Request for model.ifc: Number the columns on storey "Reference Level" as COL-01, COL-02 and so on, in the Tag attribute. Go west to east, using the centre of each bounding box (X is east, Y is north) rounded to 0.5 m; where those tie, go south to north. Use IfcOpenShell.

First a look at what the model holds.

```python
import ifcopenshell
import ifcopenshell.util.element
import ifcopenshell.util.placement

model = ifcopenshell.open("model.ifc")
print(model.schema)
storey = next(s for s in model.by_type("IfcBuildingStorey") if s.Name == "Reference Level")
columns = [e for e in ifcopenshell.util.element.get_decomposition(storey) if e.is_a("IfcColumn")]
for e in sorted(columns, key=lambda e: e.id()):
    origin = ifcopenshell.util.placement.get_local_placement(e.ObjectPlacement)[:3, 3]
    print(e.id(), e.Tag, e.Name, origin.round(2) + 0.0, sep=" | ")
```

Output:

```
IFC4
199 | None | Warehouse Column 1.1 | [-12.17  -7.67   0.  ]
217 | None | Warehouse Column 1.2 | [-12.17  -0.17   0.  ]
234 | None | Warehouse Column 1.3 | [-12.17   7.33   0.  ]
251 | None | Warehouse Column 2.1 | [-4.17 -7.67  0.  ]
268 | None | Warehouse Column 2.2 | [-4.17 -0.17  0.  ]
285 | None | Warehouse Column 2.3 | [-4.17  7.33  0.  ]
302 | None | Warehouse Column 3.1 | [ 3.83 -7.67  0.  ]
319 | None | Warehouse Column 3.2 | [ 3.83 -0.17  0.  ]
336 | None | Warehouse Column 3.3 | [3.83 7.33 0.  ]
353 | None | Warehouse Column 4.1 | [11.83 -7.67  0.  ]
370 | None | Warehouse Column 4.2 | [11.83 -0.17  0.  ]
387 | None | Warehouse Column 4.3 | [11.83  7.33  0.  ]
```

```python
import ifcopenshell
import ifcopenshell.geom
import ifcopenshell.util.element
import ifcopenshell.util.shape

model = ifcopenshell.open("model.ifc")
settings = ifcopenshell.geom.settings()
settings.set("use-world-coords", True)


def centre(element):
    shape = ifcopenshell.geom.create_shape(settings, element)
    return ifcopenshell.util.shape.get_bbox_centroid(shape.geometry)


storey = next(s for s in model.by_type("IfcBuildingStorey") if s.Name == "Reference Level")
columns = [e for e in ifcopenshell.util.element.get_decomposition(storey) if e.is_a("IfcColumn")]

# Insertion points can sit at a corner or the storey origin, so sort by the geometry (in metres).
centres = {e: centre(e) for e in columns}
columns.sort(key=lambda e: (round(centres[e][0] / 0.5), centres[e][1]))

for i, e in enumerate(columns, start=1):
    number = f"COL-{i:02d}"
    e.Tag = number
    print(e.id(), number)

model.write("model_updated.ifc")
```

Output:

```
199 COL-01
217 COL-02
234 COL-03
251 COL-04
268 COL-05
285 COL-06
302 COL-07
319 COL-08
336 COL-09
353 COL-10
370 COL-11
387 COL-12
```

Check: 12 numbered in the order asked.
